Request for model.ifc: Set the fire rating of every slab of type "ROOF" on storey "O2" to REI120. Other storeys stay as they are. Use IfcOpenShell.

First a look at what the model holds.

```python
import ifcopenshell
import ifcopenshell.util.element

model = ifcopenshell.open("model.ifc")
print(model.schema)
storey = next(s for s in model.by_type("IfcBuildingStorey") if s.Name == "O2")
slabs = [e for e in ifcopenshell.util.element.get_decomposition(storey) if e.is_a("IfcSlab")]
seen = {}
for e in slabs:
    element_type = ifcopenshell.util.element.get_type(e)
    key = (element_type.Name if element_type != e and element_type else None, ifcopenshell.util.element.get_pset(e, "Pset_SlabCommon", "FireRating"))
    seen[key] = seen.get(key, 0) + 1
for (name, value), count in sorted(seen.items(), key=str):
    print(count, "x", name, "|", value)
```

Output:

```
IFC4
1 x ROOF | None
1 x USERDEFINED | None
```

```python
import ifcopenshell
import ifcopenshell.api.pset
import ifcopenshell.util.element

model = ifcopenshell.open("model.ifc")

storey = next(s for s in model.by_type("IfcBuildingStorey") if s.Name == "O2")
slabs = [e for e in ifcopenshell.util.element.get_decomposition(storey) if e.is_a("IfcSlab")]

count = 0
for e in slabs:
    element_type = ifcopenshell.util.element.get_type(e)
    if element_type in (None, e) or element_type.Name != "ROOF":
        continue
    # add_pset returns the element's existing set when there is one.
    pset = ifcopenshell.api.pset.add_pset(model, product=e, name="Pset_SlabCommon")
    ifcopenshell.api.pset.edit_pset(model, pset=pset, properties={"FireRating": "REI120"})
    count += 1

print(count, "slabs updated")

model.write("model-out.ifc")
```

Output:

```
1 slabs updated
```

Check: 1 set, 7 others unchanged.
